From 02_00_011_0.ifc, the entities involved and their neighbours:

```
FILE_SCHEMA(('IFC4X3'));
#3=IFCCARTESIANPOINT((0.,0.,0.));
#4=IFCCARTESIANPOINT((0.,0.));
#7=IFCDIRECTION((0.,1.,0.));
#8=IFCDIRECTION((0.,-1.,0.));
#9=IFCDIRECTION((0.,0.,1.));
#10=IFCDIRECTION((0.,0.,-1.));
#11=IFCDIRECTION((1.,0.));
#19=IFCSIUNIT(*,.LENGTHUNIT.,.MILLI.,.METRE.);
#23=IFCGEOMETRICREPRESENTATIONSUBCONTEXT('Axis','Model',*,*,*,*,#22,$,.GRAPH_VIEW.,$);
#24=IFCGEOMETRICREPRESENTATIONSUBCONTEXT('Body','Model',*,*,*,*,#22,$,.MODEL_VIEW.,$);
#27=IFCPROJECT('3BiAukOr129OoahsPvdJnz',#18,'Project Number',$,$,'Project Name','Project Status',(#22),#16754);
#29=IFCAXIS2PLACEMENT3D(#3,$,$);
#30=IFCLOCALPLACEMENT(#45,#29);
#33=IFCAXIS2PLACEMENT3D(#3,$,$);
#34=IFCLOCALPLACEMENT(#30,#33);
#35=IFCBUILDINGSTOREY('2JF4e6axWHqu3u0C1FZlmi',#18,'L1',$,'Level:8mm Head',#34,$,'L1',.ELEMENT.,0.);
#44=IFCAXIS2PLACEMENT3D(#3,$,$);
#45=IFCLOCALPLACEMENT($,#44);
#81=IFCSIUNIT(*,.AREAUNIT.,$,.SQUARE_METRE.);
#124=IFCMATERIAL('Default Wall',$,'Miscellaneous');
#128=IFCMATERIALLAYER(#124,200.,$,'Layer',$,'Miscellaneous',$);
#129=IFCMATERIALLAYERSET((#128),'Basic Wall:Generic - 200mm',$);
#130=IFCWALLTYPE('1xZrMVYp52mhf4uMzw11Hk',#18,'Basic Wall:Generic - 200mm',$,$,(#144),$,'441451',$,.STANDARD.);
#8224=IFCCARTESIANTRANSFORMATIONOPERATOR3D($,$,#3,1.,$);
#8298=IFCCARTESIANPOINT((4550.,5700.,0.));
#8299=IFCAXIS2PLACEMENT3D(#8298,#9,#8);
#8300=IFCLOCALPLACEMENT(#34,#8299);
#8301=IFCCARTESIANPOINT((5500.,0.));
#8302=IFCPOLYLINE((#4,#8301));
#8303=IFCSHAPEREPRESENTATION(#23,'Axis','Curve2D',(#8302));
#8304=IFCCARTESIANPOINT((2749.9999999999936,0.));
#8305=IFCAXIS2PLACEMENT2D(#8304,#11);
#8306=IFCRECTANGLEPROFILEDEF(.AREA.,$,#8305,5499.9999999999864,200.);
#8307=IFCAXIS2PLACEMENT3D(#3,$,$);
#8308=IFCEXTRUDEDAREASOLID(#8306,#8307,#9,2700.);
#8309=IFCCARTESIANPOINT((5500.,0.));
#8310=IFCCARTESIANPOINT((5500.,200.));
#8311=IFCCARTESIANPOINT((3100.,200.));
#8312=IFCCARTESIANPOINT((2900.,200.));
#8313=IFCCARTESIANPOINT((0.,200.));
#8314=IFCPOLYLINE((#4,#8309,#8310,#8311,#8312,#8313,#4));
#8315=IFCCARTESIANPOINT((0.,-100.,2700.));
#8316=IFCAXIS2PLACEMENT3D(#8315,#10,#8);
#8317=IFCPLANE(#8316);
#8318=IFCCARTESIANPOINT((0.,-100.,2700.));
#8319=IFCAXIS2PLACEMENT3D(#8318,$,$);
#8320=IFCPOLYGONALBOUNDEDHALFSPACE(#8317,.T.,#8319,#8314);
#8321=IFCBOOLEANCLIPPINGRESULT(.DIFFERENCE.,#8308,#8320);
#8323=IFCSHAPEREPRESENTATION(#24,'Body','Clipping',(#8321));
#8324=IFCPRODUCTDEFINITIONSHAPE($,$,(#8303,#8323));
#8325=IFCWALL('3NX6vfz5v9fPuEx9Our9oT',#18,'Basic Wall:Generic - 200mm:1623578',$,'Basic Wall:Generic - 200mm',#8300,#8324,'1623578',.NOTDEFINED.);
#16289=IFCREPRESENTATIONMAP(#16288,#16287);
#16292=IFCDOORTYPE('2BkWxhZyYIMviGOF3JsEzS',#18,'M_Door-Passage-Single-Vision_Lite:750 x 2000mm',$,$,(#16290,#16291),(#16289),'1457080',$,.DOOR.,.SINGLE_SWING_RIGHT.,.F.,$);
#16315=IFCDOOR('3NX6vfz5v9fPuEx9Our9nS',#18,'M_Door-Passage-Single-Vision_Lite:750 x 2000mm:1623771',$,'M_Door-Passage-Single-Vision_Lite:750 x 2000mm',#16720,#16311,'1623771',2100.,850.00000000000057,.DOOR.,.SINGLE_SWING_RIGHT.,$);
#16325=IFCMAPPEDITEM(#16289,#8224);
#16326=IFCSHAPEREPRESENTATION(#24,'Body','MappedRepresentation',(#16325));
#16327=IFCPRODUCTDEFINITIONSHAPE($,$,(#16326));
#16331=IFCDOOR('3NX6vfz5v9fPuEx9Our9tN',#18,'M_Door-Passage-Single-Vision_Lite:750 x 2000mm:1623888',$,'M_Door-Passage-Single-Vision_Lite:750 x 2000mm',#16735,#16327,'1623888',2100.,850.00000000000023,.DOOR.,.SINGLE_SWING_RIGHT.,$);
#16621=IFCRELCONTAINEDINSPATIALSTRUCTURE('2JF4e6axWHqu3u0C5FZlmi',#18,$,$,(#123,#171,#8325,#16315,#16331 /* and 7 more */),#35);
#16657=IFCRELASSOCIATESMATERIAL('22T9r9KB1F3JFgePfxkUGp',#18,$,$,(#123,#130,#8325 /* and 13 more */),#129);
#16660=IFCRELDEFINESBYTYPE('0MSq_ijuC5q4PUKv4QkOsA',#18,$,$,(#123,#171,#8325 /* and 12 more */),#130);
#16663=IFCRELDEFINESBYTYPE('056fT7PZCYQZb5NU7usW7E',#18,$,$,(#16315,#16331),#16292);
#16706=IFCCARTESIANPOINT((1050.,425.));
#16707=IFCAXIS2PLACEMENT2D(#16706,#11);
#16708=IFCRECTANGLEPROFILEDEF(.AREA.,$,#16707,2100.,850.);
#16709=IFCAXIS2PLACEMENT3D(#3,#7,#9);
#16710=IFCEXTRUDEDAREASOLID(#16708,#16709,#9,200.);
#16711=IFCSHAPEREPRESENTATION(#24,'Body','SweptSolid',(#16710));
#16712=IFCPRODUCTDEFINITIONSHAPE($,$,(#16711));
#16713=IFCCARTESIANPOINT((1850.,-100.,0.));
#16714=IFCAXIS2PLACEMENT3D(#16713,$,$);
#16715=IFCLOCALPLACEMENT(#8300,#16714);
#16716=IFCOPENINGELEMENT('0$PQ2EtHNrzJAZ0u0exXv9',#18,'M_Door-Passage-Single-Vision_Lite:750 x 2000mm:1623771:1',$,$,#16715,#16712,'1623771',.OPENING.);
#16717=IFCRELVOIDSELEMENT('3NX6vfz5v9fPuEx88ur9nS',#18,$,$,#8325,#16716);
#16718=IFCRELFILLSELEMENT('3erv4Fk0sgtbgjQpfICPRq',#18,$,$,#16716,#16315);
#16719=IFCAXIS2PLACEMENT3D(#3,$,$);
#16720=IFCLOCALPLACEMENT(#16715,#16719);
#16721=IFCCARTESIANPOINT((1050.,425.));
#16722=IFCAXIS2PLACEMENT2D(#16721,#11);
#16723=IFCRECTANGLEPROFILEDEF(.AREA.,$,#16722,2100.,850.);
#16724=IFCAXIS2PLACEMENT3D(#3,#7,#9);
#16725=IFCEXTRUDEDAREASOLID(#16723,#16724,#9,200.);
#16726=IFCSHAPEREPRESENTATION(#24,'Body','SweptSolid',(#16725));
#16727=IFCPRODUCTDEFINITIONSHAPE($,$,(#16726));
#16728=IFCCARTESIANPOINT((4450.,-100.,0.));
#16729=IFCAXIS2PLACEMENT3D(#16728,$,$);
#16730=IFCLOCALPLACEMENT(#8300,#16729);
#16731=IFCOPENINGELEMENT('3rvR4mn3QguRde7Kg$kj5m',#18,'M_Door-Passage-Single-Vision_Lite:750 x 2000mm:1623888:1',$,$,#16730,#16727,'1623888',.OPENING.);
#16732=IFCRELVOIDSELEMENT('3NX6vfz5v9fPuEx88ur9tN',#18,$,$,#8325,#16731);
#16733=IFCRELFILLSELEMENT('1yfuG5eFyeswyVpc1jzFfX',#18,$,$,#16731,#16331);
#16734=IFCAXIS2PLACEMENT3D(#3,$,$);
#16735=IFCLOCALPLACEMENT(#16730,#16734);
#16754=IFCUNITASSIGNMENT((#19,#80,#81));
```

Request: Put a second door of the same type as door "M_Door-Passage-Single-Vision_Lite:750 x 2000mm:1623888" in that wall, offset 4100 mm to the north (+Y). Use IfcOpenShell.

```python
import ifcopenshell
import ifcopenshell.api.feature
import ifcopenshell.api.geometry
import ifcopenshell.api.root
import ifcopenshell.geom
import ifcopenshell.util.element
import ifcopenshell.util.placement
import ifcopenshell.util.shape
import ifcopenshell.util.unit

model = ifcopenshell.open("02_00_011_0.ifc")
unit_scale = ifcopenshell.util.unit.calculate_unit_scale(model)
settings = ifcopenshell.geom.settings()


def volume(element):
    """Net volume in cubic metres, openings subtracted."""
    shape = ifcopenshell.geom.create_shape(settings, element)
    return ifcopenshell.util.shape.get_volume(shape.geometry)


def reuse_history(source, copy):
    """copy_class also copies each property set's owner history, people and application; keep the originals."""
    for rel in copy.IsDefinedBy:
        if rel.is_a("IfcRelDefinesByProperties") and (history := rel.RelatingPropertyDefinition.OwnerHistory):
            rel.RelatingPropertyDefinition.OwnerHistory = source.OwnerHistory
            ifcopenshell.util.element.remove_deep2(model, history)


door = model.by_guid("3NX6vfz5v9fPuEx9Our9tN")
opening = door.FillsVoids[0].RelatingOpeningElement
wall = opening.VoidsElements[0].RelatingBuildingElement
before = volume(wall)
shift = ifcopenshell.util.placement.get_local_placement(wall.ObjectPlacement)[:3, 0] * -4.1 / unit_scale

# copy_class copies the void relationship, type, container and properties, but no geometry.
new_opening = ifcopenshell.api.root.copy_class(model, product=opening)
new_opening.Representation = ifcopenshell.util.element.copy_deep(
    model, opening.Representation, exclude=["IfcGeometricRepresentationContext", "IfcRepresentationMap"]
)
new_opening.Name = "M_Door-Passage-Single-Vision_Lite:750 x 2000mm"
new_opening.Tag = None
new_door = ifcopenshell.api.root.copy_class(model, product=door)
new_door.Representation = ifcopenshell.util.element.copy_deep(
    model, door.Representation, exclude=["IfcGeometricRepresentationContext", "IfcRepresentationMap"]
)
new_door.Name = "M_Door-Passage-Single-Vision_Lite:750 x 2000mm"
new_door.Tag = None
reuse_history(door, new_door)
ifcopenshell.api.feature.add_filling(model, opening=new_opening, element=new_door)

for old, new in ((opening, new_opening), (door, new_door)):
    matrix = ifcopenshell.util.placement.get_local_placement(old.ObjectPlacement)
    matrix[:3, 3] += shift
    ifcopenshell.api.geometry.edit_object_placement(model, product=new, matrix=matrix, is_si=False)

after = volume(wall)

print(f"wall volume {before:.3f} -> {after:.3f} m3")

model.write("02_00_011_0_rev.ifc")
```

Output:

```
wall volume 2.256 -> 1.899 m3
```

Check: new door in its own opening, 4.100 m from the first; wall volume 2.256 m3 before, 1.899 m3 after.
